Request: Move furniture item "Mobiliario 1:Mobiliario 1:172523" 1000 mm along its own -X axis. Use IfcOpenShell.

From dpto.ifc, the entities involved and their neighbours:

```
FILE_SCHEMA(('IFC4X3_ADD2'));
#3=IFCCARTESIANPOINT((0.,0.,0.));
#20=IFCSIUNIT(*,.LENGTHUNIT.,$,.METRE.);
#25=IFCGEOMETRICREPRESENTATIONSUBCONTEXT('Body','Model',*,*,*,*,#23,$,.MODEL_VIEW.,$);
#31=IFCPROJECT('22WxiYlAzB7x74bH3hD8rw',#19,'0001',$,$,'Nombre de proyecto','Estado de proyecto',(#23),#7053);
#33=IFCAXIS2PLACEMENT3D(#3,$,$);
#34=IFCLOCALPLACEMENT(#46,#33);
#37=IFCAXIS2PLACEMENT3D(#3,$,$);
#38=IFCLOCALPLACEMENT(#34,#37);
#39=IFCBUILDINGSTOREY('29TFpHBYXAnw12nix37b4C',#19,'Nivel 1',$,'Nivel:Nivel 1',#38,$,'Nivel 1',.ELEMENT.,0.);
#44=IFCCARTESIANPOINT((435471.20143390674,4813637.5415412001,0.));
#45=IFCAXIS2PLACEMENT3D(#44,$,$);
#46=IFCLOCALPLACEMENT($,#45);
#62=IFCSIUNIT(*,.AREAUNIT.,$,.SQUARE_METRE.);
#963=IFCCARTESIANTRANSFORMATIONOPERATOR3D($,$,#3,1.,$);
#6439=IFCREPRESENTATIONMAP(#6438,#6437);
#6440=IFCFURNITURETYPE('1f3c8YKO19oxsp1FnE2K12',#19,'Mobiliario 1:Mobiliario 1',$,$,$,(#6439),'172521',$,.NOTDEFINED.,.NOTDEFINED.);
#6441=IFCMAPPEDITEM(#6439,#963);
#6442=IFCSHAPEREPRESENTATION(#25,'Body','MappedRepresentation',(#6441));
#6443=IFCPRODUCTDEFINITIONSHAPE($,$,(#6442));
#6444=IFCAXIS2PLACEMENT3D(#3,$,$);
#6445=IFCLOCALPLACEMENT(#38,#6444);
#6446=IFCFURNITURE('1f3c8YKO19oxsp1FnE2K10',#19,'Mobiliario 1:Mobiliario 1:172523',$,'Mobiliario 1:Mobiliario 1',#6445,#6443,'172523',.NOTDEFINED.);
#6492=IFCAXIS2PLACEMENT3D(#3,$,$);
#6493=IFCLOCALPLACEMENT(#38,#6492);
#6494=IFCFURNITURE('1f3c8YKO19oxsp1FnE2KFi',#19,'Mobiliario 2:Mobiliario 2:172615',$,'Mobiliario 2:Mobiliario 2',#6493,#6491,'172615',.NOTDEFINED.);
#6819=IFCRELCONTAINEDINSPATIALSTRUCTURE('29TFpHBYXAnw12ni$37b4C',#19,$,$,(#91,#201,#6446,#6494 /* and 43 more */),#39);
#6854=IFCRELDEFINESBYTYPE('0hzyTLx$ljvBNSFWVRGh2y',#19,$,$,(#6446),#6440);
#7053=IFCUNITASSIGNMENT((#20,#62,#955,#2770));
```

```python
import ifcopenshell
import ifcopenshell.api.geometry
import ifcopenshell.util.placement

model = ifcopenshell.open("dpto.ifc")

item = model.by_guid("1f3c8YKO19oxsp1FnE2K10")
matrix = ifcopenshell.util.placement.get_local_placement(item.ObjectPlacement)
matrix[:3, 3] -= matrix[:3, 0] * 1.0
ifcopenshell.api.geometry.edit_object_placement(model, product=item, matrix=matrix, is_si=False)

print(ifcopenshell.util.placement.get_local_placement(item.ObjectPlacement).round(3) + 0.0)

model.write("dpto_updated.ifc")
```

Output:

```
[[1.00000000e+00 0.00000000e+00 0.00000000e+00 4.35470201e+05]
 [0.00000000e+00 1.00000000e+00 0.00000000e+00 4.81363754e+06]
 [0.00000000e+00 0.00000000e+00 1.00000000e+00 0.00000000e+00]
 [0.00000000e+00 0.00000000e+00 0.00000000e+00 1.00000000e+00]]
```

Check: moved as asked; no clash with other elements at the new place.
